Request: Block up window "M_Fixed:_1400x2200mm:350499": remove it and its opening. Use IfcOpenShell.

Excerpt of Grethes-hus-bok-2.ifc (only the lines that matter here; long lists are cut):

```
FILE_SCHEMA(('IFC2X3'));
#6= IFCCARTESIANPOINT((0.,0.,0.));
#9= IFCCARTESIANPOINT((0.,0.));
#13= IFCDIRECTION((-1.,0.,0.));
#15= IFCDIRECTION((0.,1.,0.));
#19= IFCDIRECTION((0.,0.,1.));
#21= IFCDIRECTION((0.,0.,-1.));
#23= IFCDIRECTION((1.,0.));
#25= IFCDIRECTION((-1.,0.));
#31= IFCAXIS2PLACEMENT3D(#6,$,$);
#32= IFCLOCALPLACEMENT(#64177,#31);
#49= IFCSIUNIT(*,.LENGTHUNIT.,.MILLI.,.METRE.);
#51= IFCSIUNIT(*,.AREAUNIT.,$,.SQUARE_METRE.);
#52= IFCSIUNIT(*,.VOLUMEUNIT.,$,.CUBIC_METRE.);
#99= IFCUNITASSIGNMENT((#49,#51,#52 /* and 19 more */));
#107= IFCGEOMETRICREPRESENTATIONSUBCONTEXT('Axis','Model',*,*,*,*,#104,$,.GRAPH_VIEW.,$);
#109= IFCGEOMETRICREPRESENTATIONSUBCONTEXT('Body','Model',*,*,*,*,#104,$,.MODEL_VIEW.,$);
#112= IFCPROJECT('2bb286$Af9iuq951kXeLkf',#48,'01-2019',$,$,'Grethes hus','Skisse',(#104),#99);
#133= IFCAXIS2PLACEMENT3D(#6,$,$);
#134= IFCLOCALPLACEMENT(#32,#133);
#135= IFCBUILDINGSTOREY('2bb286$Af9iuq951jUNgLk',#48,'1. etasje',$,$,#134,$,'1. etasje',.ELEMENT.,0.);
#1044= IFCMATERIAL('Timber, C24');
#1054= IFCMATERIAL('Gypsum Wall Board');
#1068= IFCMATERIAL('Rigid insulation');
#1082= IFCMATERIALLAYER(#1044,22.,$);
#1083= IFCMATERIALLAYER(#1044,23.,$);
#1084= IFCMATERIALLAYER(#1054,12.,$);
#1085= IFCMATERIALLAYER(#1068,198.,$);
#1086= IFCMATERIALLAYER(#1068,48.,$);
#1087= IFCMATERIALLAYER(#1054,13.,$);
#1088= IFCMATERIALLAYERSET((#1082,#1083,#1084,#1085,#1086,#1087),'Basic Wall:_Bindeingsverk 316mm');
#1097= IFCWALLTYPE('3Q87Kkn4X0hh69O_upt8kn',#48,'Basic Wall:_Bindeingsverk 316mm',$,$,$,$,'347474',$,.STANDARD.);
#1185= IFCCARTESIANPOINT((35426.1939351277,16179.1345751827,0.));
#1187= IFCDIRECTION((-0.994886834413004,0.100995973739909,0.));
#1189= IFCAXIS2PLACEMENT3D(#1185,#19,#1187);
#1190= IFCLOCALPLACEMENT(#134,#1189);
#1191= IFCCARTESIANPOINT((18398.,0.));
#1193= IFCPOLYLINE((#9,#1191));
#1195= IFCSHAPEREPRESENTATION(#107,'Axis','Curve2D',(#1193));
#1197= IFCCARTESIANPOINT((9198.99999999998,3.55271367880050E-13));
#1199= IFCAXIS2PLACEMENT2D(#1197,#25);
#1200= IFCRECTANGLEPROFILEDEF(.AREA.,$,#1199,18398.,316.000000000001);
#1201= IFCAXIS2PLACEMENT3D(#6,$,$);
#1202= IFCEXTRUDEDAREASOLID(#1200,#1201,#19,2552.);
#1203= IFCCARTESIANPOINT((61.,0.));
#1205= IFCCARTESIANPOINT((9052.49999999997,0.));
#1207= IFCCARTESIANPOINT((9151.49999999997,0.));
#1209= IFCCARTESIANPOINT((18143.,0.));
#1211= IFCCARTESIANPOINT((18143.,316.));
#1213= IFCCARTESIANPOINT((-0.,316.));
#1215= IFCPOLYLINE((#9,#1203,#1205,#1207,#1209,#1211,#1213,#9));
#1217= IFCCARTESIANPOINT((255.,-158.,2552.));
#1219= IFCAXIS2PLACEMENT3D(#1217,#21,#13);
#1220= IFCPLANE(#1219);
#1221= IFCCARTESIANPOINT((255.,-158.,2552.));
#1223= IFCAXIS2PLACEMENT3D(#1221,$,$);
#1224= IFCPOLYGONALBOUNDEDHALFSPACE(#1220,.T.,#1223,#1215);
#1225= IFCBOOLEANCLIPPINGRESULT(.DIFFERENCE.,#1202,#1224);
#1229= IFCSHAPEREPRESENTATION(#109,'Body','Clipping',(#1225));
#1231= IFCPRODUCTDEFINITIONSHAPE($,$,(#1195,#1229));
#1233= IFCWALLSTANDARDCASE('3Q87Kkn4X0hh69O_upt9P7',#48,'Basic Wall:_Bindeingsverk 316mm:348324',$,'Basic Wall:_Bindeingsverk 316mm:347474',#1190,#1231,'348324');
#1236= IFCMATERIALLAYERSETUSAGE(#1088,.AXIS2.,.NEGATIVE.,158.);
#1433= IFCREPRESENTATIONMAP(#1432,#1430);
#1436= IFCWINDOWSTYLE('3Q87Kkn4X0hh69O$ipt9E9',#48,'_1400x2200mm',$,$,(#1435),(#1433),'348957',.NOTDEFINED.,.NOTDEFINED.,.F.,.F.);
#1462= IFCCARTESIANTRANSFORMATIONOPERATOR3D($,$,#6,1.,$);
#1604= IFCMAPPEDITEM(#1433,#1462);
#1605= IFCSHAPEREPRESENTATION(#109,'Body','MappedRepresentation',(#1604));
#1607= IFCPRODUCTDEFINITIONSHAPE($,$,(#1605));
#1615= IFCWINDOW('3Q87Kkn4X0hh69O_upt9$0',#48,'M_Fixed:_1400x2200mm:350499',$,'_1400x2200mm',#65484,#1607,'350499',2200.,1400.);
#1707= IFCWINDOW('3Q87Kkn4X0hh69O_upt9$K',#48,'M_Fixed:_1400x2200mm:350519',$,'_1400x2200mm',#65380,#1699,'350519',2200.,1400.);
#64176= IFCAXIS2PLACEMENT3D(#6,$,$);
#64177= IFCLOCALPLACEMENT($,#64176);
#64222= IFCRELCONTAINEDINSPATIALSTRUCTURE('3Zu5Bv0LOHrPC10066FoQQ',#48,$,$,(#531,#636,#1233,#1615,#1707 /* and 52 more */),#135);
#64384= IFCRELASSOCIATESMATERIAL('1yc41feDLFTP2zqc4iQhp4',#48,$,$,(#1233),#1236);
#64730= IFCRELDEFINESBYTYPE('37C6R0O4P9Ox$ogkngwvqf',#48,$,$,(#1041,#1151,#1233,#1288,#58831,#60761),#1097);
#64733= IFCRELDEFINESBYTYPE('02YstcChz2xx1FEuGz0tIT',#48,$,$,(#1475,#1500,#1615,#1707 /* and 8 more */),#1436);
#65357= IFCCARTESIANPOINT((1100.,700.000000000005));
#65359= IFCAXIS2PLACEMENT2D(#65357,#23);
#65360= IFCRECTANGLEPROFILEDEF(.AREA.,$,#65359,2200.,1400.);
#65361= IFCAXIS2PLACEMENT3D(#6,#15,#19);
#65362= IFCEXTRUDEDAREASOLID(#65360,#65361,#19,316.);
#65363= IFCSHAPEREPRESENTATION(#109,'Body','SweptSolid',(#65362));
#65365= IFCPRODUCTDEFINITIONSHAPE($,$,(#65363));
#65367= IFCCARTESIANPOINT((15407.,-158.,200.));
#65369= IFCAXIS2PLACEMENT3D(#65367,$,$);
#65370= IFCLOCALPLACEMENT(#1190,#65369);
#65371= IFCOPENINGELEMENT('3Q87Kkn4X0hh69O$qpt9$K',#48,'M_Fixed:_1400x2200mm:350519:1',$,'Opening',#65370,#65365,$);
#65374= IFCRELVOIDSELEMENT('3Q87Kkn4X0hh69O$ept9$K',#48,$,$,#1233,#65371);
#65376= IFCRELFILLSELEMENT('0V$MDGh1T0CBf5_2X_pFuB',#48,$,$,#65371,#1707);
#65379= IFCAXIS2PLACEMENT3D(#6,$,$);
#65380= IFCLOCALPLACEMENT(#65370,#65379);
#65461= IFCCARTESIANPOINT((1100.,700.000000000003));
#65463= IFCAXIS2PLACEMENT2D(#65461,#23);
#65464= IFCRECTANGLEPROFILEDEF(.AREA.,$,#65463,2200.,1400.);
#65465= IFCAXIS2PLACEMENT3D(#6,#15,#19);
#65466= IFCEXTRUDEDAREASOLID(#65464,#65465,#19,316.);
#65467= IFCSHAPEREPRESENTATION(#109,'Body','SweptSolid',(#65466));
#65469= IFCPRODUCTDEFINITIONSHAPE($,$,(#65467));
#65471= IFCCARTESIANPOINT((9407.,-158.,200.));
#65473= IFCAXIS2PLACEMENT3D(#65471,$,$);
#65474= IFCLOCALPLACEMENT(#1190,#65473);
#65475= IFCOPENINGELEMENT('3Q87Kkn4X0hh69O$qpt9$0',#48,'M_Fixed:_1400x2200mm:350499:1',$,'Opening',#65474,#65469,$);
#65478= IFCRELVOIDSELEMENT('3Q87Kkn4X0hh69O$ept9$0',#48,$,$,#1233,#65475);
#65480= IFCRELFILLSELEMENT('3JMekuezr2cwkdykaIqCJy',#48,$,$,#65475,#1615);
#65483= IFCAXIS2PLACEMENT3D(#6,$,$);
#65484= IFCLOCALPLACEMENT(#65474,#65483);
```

```python
import ifcopenshell
import ifcopenshell.api.feature
import ifcopenshell.api.root
import ifcopenshell.geom
import ifcopenshell.util.shape

model = ifcopenshell.open("Grethes-hus-bok-2.ifc")
settings = ifcopenshell.geom.settings()


def volume(element):
    """Net volume in cubic metres, openings subtracted."""
    shape = ifcopenshell.geom.create_shape(settings, element)
    return ifcopenshell.util.shape.get_volume(shape.geometry)


window = model.by_guid("3Q87Kkn4X0hh69O_upt9$0")
opening = window.FillsVoids[0].RelatingOpeningElement
wall = opening.VoidsElements[0].RelatingBuildingElement
before = volume(wall)

ifcopenshell.api.root.remove_product(model, product=window)
ifcopenshell.api.feature.remove_feature(model, feature=opening)

after = volume(wall)

print(f"wall volume {before:.3f} -> {after:.3f} m3")

model.write("Grethes-hus-bok-2_rev.ifc")
```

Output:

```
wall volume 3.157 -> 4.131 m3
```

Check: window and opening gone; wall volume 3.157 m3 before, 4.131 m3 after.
